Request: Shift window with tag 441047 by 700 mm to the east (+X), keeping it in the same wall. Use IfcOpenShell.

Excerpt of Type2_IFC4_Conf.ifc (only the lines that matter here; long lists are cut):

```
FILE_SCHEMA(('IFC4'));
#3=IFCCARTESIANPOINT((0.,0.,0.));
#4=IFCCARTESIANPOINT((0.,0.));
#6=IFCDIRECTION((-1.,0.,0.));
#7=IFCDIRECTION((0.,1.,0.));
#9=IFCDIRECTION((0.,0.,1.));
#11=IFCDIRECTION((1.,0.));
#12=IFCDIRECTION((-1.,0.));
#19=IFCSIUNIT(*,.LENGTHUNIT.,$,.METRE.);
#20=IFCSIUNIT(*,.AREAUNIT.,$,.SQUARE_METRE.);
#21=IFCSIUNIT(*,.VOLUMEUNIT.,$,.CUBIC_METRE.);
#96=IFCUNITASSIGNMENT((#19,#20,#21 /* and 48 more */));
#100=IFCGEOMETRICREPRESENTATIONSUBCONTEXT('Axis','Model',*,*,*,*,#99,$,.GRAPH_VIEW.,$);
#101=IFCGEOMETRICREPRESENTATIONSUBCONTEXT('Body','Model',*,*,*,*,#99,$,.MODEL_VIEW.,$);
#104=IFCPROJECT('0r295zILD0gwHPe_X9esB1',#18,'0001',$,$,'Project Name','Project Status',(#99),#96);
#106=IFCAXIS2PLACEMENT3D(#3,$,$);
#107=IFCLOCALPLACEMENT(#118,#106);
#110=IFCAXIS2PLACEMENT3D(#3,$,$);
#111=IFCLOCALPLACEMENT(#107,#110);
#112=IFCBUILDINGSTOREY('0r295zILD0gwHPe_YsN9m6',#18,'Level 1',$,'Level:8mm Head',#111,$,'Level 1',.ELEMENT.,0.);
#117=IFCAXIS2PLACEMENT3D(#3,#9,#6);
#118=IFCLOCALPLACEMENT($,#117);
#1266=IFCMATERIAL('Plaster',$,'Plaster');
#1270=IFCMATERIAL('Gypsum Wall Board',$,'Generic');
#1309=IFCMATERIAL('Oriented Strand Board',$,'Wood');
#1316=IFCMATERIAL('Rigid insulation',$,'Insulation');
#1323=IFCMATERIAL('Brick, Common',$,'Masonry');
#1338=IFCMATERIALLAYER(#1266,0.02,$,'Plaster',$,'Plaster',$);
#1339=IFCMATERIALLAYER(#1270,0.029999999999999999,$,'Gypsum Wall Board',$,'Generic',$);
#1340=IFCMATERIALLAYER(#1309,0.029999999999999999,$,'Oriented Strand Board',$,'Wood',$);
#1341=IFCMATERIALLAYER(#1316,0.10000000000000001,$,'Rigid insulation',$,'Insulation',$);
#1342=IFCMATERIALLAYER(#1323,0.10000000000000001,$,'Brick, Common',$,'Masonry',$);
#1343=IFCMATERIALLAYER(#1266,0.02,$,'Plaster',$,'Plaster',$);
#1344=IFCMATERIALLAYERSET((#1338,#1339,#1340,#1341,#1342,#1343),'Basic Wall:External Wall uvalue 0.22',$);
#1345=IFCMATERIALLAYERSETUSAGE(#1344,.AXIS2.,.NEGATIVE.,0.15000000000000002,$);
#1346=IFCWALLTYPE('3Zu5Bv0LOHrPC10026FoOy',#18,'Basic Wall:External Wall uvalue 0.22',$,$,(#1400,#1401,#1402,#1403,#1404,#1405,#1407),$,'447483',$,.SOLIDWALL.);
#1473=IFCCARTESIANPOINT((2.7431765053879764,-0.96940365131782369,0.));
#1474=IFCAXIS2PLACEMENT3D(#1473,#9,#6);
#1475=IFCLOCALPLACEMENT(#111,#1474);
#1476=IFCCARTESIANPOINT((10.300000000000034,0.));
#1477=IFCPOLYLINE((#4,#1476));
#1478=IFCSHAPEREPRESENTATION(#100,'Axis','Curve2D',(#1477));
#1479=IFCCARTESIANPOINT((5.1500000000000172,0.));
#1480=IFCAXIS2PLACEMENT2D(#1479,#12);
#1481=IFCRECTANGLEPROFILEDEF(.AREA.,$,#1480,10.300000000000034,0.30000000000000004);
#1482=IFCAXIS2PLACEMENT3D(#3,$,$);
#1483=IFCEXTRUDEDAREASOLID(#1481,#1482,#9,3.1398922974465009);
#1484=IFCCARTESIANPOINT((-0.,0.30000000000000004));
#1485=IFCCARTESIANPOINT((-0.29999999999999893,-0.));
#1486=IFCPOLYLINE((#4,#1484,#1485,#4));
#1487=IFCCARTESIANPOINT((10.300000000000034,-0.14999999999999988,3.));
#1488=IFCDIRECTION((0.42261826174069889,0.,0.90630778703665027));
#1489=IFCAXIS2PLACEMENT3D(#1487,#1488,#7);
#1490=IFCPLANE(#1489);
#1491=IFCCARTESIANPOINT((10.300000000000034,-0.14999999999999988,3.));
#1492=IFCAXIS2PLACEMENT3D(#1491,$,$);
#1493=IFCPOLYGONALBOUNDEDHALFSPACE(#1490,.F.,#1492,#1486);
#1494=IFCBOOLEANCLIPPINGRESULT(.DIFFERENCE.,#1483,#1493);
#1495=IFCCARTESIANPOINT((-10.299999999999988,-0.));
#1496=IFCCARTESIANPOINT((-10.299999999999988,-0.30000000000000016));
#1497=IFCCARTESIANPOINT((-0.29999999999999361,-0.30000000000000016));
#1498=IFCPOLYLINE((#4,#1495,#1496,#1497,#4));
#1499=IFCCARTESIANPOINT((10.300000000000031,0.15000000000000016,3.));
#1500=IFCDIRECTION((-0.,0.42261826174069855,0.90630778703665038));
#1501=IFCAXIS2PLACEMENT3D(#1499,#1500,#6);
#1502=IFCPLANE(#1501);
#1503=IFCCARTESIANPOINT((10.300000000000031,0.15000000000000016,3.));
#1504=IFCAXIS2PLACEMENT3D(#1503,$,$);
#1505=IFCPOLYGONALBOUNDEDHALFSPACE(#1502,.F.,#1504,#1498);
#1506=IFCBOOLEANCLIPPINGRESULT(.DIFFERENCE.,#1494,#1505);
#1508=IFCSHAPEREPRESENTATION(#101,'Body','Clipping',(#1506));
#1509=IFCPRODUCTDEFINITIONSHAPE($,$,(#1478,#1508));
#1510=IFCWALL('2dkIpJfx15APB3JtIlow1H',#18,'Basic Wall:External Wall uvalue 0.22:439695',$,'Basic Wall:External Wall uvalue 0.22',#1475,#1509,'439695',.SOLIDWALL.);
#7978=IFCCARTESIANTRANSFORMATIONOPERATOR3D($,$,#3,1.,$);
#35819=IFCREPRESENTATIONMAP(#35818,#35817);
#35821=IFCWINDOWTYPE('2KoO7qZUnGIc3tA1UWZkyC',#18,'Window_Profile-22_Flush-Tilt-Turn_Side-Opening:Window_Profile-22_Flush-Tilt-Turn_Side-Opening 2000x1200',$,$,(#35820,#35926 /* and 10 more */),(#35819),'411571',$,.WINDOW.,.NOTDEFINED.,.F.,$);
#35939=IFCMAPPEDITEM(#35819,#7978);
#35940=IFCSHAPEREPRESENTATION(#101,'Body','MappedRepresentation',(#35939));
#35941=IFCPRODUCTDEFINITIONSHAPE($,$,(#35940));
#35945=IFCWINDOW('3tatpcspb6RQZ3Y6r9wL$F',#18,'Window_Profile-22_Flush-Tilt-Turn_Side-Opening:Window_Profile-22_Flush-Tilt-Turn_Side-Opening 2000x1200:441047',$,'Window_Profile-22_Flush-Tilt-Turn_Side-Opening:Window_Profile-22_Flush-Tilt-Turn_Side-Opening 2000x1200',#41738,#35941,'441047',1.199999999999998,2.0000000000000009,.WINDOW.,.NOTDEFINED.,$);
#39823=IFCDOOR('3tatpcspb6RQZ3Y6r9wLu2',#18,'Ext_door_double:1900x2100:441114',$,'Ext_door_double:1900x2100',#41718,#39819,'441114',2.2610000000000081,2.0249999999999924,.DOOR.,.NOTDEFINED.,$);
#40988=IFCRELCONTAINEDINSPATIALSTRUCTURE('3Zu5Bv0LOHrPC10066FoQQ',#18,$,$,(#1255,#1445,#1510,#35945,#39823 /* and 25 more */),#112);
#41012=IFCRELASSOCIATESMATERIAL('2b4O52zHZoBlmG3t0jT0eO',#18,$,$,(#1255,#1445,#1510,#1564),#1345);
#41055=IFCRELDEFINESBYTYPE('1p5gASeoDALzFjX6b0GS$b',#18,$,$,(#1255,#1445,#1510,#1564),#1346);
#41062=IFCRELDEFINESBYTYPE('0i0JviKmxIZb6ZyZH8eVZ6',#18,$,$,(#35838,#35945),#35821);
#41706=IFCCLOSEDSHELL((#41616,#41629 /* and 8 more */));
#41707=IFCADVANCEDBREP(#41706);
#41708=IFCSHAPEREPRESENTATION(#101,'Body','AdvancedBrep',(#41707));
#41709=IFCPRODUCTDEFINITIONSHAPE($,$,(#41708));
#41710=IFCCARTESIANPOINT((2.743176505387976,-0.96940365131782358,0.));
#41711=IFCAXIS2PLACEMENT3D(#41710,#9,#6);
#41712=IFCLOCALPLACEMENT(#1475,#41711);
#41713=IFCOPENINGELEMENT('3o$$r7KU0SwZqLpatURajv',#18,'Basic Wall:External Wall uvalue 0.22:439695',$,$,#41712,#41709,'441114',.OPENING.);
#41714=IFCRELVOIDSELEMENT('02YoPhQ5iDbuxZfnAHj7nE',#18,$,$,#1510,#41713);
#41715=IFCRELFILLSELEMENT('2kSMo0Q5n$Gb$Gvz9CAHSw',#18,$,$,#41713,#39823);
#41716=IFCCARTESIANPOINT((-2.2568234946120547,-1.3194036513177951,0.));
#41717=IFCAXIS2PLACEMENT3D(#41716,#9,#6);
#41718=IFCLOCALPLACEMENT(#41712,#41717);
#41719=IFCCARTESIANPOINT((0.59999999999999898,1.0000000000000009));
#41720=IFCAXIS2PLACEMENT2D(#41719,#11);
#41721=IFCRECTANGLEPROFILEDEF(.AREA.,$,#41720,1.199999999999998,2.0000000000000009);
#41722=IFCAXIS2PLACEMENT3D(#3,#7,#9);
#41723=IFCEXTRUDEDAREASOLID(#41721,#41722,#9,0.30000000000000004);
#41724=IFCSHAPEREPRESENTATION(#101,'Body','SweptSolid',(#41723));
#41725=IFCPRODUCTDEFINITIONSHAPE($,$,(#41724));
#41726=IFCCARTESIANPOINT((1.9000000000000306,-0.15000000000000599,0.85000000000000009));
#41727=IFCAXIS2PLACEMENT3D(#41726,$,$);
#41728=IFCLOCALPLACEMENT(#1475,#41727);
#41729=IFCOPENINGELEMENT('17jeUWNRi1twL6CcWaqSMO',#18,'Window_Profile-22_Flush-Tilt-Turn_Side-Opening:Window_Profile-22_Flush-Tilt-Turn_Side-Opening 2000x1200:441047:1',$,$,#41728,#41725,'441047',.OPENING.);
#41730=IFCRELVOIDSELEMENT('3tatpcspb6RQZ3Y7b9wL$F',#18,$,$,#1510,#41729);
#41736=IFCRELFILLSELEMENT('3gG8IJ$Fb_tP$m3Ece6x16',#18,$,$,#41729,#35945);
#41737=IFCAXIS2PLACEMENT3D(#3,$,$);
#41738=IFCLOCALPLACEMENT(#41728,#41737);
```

```python
import ifcopenshell
import ifcopenshell.api.geometry
import ifcopenshell.util.placement
import ifcopenshell.util.unit

model = ifcopenshell.open("Type2_IFC4_Conf.ifc")
unit_scale = ifcopenshell.util.unit.calculate_unit_scale(model)

window = model.by_guid("3tatpcspb6RQZ3Y6r9wL$F")
opening = window.FillsVoids[0].RelatingOpeningElement
wall = opening.VoidsElements[0].RelatingBuildingElement

wall_matrix = ifcopenshell.util.placement.get_local_placement(wall.ObjectPlacement)
shift = wall_matrix[:3, 0] * 0.7 / unit_scale
before = ifcopenshell.util.placement.get_local_placement(window.ObjectPlacement)[:3, 3].copy()

# The window is placed relative to its opening, so it follows when the opening moves.
matrix = ifcopenshell.util.placement.get_local_placement(opening.ObjectPlacement)
matrix[:3, 3] += shift
ifcopenshell.api.geometry.edit_object_placement(
    model, product=opening, matrix=matrix, is_si=False, should_transform_children=True
)

after = ifcopenshell.util.placement.get_local_placement(window.ObjectPlacement)[:3, 3]
print("window moved by", (after - before).round(3) + 0.0)

model.write("Type2_IFC4_Conf_edited.ifc")
```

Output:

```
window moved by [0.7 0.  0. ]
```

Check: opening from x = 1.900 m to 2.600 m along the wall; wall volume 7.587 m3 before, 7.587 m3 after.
